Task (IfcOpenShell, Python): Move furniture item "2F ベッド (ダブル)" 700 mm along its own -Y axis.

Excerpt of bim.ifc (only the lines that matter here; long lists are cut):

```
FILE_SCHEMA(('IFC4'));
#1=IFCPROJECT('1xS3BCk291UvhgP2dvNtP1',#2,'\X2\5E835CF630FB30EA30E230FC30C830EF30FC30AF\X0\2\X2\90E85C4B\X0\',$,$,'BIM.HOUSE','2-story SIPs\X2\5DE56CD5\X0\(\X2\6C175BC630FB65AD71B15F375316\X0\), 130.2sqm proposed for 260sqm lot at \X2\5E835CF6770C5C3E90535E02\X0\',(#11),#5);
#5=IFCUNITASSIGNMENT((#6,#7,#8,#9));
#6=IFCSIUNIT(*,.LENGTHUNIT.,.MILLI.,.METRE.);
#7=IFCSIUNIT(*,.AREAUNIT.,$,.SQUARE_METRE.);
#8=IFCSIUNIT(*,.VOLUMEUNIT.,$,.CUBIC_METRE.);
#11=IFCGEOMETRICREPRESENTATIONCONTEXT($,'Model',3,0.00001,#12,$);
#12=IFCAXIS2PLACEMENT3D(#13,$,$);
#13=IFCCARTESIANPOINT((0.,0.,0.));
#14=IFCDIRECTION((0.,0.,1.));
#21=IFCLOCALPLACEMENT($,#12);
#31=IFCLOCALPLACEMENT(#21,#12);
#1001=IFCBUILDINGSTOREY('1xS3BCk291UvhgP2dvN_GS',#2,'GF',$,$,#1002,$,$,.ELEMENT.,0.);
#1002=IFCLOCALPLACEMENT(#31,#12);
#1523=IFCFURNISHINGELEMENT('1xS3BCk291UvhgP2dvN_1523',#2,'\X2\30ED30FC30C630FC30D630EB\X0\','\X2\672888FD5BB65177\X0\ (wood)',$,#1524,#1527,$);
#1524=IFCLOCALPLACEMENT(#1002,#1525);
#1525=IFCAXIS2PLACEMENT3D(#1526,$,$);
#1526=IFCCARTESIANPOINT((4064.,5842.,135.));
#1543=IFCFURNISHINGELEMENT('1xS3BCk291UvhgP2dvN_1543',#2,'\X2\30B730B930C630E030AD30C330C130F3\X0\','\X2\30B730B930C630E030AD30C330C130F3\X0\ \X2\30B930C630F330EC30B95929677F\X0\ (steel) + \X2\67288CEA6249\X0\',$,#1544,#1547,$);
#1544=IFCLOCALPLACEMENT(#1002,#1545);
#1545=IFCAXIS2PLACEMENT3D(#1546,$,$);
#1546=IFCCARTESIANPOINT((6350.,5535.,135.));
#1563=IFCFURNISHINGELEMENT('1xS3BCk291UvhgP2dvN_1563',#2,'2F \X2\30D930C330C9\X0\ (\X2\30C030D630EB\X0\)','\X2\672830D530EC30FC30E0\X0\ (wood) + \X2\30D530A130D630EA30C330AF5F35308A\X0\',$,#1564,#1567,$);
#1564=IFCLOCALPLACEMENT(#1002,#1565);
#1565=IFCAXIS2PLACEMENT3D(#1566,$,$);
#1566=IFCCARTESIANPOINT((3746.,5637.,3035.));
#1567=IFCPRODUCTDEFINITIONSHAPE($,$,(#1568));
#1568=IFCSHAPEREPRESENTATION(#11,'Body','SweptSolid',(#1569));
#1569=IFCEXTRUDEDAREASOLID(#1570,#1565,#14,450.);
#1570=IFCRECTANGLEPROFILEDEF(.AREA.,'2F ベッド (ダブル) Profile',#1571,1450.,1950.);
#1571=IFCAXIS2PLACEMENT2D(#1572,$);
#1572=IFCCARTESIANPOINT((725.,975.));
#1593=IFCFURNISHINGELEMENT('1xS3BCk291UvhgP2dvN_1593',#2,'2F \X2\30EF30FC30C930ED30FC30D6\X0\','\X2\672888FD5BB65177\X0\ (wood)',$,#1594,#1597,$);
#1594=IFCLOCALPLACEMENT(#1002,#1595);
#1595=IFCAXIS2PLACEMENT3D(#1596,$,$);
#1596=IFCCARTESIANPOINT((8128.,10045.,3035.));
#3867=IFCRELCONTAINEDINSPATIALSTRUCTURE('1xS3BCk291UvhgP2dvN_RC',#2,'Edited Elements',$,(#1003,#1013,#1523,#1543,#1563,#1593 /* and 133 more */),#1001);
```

```python
import ifcopenshell
import ifcopenshell.api.geometry
import ifcopenshell.util.placement
import ifcopenshell.util.unit

model = ifcopenshell.open("bim.ifc")
unit_scale = ifcopenshell.util.unit.calculate_unit_scale(model)

item = model.by_id(1563)
matrix = ifcopenshell.util.placement.get_local_placement(item.ObjectPlacement)
matrix[:3, 3] -= matrix[:3, 1] * 0.7 / unit_scale
ifcopenshell.api.geometry.edit_object_placement(model, product=item, matrix=matrix, is_si=False)

print(ifcopenshell.util.placement.get_local_placement(item.ObjectPlacement).round(3) + 0.0)

model.write("bim_v2.ifc")
```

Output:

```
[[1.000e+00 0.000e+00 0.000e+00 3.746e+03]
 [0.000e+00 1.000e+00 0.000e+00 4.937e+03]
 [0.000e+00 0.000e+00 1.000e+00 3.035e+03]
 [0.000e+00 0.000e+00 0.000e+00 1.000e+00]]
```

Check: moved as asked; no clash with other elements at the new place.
